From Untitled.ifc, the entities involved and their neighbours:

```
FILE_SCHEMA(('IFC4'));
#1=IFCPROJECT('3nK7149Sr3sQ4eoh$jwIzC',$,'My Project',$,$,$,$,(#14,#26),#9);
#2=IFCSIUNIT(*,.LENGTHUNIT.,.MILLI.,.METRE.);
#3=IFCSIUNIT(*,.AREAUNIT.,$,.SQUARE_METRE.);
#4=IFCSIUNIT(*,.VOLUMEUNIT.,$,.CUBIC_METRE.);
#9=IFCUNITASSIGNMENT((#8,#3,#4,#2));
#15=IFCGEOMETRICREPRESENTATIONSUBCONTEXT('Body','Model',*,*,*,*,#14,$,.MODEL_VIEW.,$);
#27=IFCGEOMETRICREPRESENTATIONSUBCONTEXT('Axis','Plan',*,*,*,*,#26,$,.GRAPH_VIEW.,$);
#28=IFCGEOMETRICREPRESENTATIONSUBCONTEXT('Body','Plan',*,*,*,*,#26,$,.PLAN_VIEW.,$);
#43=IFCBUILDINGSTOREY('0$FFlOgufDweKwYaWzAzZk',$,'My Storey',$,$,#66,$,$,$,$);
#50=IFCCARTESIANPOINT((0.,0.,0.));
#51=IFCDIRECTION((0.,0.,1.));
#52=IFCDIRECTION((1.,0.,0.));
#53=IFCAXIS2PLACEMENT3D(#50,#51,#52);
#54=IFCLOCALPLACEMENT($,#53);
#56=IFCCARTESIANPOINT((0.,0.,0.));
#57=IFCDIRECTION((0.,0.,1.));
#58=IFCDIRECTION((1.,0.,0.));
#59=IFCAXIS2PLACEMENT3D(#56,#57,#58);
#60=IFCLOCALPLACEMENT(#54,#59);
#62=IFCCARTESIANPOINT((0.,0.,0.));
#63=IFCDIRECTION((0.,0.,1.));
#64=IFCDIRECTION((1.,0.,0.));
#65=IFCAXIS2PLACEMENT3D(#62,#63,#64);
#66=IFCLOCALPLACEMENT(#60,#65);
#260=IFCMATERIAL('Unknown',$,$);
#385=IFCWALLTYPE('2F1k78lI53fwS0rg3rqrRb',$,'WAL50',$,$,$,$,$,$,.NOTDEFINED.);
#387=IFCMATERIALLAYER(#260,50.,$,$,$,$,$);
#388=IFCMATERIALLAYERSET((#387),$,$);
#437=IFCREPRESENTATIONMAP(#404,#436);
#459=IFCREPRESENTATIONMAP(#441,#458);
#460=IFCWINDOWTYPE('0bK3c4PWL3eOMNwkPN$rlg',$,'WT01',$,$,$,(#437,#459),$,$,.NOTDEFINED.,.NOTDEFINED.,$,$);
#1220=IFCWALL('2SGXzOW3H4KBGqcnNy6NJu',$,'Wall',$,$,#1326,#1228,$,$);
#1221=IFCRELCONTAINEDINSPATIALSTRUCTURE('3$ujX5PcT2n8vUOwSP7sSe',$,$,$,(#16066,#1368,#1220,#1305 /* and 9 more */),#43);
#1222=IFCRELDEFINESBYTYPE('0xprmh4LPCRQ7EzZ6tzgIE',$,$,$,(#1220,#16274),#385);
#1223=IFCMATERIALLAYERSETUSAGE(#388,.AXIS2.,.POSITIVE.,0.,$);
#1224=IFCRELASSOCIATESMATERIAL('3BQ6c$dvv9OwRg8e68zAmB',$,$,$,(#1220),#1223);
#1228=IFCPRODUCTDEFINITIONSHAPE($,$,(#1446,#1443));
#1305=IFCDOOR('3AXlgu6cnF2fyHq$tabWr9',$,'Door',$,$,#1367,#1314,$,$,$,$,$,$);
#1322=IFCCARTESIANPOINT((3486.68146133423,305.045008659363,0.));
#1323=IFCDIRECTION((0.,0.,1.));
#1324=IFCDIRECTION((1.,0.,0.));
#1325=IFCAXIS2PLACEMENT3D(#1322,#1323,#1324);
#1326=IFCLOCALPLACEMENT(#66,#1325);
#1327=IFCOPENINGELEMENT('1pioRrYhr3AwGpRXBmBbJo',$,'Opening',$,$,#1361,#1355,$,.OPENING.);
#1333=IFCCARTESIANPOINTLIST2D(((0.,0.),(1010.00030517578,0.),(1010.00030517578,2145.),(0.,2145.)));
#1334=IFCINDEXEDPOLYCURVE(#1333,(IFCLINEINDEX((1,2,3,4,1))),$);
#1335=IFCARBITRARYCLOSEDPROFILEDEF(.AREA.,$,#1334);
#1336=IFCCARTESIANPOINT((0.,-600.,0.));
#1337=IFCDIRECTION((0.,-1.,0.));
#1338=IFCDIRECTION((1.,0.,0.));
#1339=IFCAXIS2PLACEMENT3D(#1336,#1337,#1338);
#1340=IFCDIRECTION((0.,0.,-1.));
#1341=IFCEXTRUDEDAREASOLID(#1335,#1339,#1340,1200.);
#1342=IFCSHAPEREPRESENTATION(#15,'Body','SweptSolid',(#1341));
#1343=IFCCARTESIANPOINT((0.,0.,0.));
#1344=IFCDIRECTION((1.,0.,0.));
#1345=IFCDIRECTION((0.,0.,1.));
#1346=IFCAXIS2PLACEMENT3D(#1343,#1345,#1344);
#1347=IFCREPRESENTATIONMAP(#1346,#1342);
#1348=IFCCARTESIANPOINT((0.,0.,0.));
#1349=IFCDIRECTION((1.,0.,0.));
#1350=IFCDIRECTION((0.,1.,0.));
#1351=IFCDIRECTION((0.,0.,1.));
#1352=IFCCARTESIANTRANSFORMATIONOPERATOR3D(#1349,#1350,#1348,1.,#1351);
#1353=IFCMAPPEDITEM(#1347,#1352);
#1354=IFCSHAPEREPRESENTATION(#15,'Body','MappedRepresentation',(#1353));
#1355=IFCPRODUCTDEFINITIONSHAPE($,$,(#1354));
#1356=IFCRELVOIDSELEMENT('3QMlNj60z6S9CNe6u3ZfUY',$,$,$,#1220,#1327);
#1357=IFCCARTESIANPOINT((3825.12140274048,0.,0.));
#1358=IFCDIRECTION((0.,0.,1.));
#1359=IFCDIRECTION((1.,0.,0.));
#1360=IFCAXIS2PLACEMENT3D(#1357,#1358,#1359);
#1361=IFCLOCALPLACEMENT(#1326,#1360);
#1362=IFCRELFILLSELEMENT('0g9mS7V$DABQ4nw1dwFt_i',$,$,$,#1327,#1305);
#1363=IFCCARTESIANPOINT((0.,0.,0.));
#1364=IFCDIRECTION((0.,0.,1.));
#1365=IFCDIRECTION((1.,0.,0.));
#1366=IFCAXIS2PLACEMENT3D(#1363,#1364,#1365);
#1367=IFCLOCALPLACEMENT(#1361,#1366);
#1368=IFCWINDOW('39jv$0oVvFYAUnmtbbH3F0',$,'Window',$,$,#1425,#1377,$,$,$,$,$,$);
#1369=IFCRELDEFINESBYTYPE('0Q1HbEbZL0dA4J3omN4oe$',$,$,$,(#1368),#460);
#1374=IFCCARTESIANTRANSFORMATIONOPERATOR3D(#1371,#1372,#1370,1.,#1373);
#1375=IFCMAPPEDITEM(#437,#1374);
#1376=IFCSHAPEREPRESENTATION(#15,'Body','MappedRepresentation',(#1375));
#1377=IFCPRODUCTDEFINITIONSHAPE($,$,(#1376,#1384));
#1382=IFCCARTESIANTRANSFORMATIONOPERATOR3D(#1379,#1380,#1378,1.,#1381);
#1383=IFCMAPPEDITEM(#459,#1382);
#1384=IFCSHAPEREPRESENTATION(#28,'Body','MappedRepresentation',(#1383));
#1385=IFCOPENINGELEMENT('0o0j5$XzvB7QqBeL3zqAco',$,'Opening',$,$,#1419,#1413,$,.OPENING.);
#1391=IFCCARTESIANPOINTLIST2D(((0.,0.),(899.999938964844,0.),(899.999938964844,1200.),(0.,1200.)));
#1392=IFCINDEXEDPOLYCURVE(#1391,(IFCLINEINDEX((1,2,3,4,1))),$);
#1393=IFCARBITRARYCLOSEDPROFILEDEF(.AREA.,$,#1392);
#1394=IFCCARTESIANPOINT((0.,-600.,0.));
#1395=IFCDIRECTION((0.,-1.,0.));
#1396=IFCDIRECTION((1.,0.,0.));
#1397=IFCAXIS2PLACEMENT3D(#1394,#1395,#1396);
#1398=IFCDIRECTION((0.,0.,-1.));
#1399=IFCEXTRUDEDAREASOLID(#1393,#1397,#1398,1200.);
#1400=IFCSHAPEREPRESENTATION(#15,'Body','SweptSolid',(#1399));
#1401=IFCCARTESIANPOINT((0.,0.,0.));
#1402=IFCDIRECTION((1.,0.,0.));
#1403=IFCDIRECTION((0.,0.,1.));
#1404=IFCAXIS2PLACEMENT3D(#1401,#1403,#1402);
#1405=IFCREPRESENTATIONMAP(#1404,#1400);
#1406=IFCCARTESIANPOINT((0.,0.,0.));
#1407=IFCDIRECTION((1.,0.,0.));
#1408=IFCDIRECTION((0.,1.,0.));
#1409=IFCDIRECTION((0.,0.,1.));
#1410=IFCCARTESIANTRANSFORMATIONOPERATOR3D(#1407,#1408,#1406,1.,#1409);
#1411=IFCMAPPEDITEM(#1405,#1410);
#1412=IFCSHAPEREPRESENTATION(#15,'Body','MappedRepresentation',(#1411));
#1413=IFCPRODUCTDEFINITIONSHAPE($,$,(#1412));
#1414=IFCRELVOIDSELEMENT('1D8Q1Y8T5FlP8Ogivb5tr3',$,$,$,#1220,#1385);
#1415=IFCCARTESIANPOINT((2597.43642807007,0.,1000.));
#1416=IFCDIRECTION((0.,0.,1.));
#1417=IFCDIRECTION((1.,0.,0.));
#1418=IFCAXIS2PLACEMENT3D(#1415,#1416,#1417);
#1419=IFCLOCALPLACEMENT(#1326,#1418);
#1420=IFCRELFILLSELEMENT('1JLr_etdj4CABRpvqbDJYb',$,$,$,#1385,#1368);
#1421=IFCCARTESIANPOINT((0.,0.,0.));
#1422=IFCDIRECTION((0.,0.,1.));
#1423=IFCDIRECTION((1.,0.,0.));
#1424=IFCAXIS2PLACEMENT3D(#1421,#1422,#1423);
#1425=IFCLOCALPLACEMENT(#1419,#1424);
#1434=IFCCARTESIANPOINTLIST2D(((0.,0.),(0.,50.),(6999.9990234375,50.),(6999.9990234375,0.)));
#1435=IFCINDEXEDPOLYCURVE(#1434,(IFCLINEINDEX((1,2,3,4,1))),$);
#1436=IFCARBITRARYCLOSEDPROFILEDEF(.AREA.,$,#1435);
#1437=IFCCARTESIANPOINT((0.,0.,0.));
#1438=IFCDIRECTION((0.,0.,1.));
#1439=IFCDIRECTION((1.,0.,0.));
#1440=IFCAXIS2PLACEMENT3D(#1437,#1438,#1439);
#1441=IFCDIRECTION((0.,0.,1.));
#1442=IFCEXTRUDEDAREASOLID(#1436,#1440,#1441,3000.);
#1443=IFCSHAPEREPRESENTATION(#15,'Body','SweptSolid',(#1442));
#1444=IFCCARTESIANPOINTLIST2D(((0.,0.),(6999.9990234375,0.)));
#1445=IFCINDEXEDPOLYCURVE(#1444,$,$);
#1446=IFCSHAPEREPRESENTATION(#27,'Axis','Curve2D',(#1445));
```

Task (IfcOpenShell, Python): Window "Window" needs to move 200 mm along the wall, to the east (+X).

```python
import ifcopenshell
import ifcopenshell.api.geometry
import ifcopenshell.util.placement
import ifcopenshell.util.unit

model = ifcopenshell.open("Untitled.ifc")
unit_scale = ifcopenshell.util.unit.calculate_unit_scale(model)

window = model.by_guid("39jv$0oVvFYAUnmtbbH3F0")
opening = window.FillsVoids[0].RelatingOpeningElement
wall = opening.VoidsElements[0].RelatingBuildingElement

wall_matrix = ifcopenshell.util.placement.get_local_placement(wall.ObjectPlacement)
shift = wall_matrix[:3, 0] * 0.2 / unit_scale
before = ifcopenshell.util.placement.get_local_placement(window.ObjectPlacement)[:3, 3].copy()

# The window is placed relative to its opening, so it follows when the opening moves.
matrix = ifcopenshell.util.placement.get_local_placement(opening.ObjectPlacement)
matrix[:3, 3] += shift
ifcopenshell.api.geometry.edit_object_placement(
    model, product=opening, matrix=matrix, is_si=False, should_transform_children=True
)

after = ifcopenshell.util.placement.get_local_placement(window.ObjectPlacement)[:3, 3]
print("window moved by", (after - before).round(3) + 0.0)

model.write("Untitled_edited.ifc")
```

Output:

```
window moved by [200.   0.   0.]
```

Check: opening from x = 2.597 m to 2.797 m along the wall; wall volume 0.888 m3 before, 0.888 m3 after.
